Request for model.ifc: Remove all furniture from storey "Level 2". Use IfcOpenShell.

First a look at what the model holds.

```python
import ifcopenshell
import ifcopenshell.util.element

model = ifcopenshell.open("model.ifc")
print(model.schema)
storey = next(s for s in model.by_type("IfcBuildingStorey") if s.Name == "Level 2")
furniture = [e for e in ifcopenshell.util.element.get_decomposition(storey) if e.is_a("IfcFurnishingElement")]
seen = {}
for e in furniture:
    element_type = ifcopenshell.util.element.get_type(e)
    name = element_type.Name if element_type not in (None, e) else None
    seen[name] = seen.get(name, 0) + 1
for name, count in sorted(seen.items(), key=str):
    print(count, "x", name)
```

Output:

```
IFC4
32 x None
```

```python
import ifcopenshell
import ifcopenshell.api.root
import ifcopenshell.util.element

model = ifcopenshell.open("model.ifc")

storey = next(s for s in model.by_type("IfcBuildingStorey") if s.Name == "Level 2")
furniture = [e for e in ifcopenshell.util.element.get_decomposition(storey) if e.is_a("IfcFurnishingElement")]

for e in furniture:
    ifcopenshell.api.root.remove_product(model, product=e)
print(len(furniture), "removed")

model.write("model-out.ifc")
```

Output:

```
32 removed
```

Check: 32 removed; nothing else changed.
